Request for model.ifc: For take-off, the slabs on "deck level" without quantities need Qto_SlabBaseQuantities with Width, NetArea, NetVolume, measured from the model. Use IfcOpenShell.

First a look at what the model holds.

```python
import ifcopenshell
import ifcopenshell.util.element
import ifcopenshell.util.unit

model = ifcopenshell.open("model.ifc")
print(model.schema)
for unit_type in ("LENGTHUNIT", "AREAUNIT", "VOLUMEUNIT"):
    print(unit_type, ifcopenshell.util.unit.calculate_unit_scale(model, unit_type))
storey = next(s for s in model.by_type("IfcBuildingStorey") if s.Name == "deck level")
slabs = [e for e in ifcopenshell.util.element.get_decomposition(storey) if e.is_a("IfcSlab")]
for e in sorted(slabs, key=lambda e: e.id()):
    print(e.id(), e.is_a(), e.Name, list(ifcopenshell.util.element.get_psets(e, qtos_only=True)), sep=" | ")
```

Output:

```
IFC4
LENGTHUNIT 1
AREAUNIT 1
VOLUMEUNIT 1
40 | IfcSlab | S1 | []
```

```python
import ifcopenshell
import ifcopenshell.api.pset
import ifcopenshell.geom
import ifcopenshell.util.element
import ifcopenshell.util.shape
import ifcopenshell.util.unit

model = ifcopenshell.open("model.ifc")
unit_scale = ifcopenshell.util.unit.calculate_unit_scale(model)
area_scale = ifcopenshell.util.unit.calculate_unit_scale(model, "AREAUNIT")
volume_scale = ifcopenshell.util.unit.calculate_unit_scale(model, "VOLUMEUNIT")
settings = ifcopenshell.geom.settings()

storey = next(s for s in model.by_type("IfcBuildingStorey") if s.Name == "deck level")
slabs = [e for e in ifcopenshell.util.element.get_decomposition(storey) if e.is_a("IfcSlab")]

for e in sorted(slabs, key=lambda e: e.id()):
    if ifcopenshell.util.element.get_psets(e, qtos_only=True, should_inherit=False):
        continue
    # Geometry comes back in metres, in the element's own axes.
    shape = ifcopenshell.geom.create_shape(settings, e)
    values = {
        "Width": ifcopenshell.util.shape.get_z(shape.geometry) / unit_scale,
        "NetArea": ifcopenshell.util.shape.get_footprint_area(shape.geometry) / area_scale,
        "NetVolume": ifcopenshell.util.shape.get_volume(shape.geometry) / volume_scale,
    }
    qto = ifcopenshell.api.pset.add_qto(model, product=e, name="Qto_SlabBaseQuantities")
    ifcopenshell.api.pset.edit_qto(model, qto=qto, properties=values)
    print(e.id(), {k: round(v, 3) for k, v in values.items()})

model.write("model-out.ifc")
```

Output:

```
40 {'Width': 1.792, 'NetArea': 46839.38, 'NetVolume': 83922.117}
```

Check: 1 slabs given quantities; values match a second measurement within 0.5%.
